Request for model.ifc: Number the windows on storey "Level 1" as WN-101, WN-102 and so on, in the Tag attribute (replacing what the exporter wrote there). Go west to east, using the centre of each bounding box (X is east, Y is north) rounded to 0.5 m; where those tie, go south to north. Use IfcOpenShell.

First a look at what the model holds.

```python
import ifcopenshell
import ifcopenshell.util.element
import ifcopenshell.util.placement

model = ifcopenshell.open("model.ifc")
print(model.schema)
storey = next(s for s in model.by_type("IfcBuildingStorey") if s.Name == "Level 1")
windows = [e for e in ifcopenshell.util.element.get_decomposition(storey) if e.is_a("IfcWindow")]
for e in sorted(windows, key=lambda e: e.id()):
    origin = ifcopenshell.util.placement.get_local_placement(e.ObjectPlacement)[:3, 3]
    print(e.id(), e.Tag, e.Name, origin.round(2) + 0.0, sep=" | ")
```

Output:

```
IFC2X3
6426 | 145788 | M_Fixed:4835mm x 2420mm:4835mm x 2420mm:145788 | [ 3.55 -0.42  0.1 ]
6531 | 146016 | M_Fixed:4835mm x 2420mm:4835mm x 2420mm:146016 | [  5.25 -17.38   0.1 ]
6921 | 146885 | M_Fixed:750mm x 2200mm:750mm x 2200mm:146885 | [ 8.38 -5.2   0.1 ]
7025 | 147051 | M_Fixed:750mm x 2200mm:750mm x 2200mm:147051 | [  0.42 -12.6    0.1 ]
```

```python
import ifcopenshell
import ifcopenshell.geom
import ifcopenshell.util.element
import ifcopenshell.util.shape

model = ifcopenshell.open("model.ifc")
settings = ifcopenshell.geom.settings()
settings.set("use-world-coords", True)


def centre(element):
    shape = ifcopenshell.geom.create_shape(settings, element)
    return ifcopenshell.util.shape.get_bbox_centroid(shape.geometry)


storey = next(s for s in model.by_type("IfcBuildingStorey") if s.Name == "Level 1")
windows = [e for e in ifcopenshell.util.element.get_decomposition(storey) if e.is_a("IfcWindow")]

# Insertion points can sit at a corner or the storey origin, so sort by the geometry (in metres).
centres = {e: centre(e) for e in windows}
windows.sort(key=lambda e: (round(centres[e][0] / 0.5), centres[e][1]))

for i, e in enumerate(windows, start=1):
    number = f"WN-1{i:02d}"
    e.Tag = number
    print(e.id(), number)

model.write("model_updated.ifc")
```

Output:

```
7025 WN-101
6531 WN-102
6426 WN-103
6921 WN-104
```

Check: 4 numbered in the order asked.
